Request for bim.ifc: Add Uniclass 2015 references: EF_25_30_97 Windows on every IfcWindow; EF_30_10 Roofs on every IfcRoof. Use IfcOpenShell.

First a look at what the model holds.

```python
import ifcopenshell

model = ifcopenshell.open("bim.ifc")
print(model.schema)
print("classifications:", [c.Name for c in model.by_type("IfcClassification")])
for ifc_class in ("IfcDoor", "IfcRoof", "IfcStair", "IfcWall", "IfcWindow"):
    print(ifc_class, len(model.by_type(ifc_class)))
```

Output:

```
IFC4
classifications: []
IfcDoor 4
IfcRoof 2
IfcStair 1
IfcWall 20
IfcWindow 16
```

```python
import ifcopenshell
import ifcopenshell.api.classification

model = ifcopenshell.open("bim.ifc")

system = ifcopenshell.api.classification.add_classification(model, classification="Uniclass 2015")

codes = {
    "IfcWindow": ("EF_25_30_97", "Windows"),
    "IfcRoof": ("EF_30_10", "Roofs"),
}
for ifc_class, (code, name) in codes.items():
    products = model.by_type(ifc_class)
    ifcopenshell.api.classification.add_reference(
        model, products=products, classification=system, identification=code, name=name
    )
    print(code, len(products))

model.write("bim_edited.ifc")
```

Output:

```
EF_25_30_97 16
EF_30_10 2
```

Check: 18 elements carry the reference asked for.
